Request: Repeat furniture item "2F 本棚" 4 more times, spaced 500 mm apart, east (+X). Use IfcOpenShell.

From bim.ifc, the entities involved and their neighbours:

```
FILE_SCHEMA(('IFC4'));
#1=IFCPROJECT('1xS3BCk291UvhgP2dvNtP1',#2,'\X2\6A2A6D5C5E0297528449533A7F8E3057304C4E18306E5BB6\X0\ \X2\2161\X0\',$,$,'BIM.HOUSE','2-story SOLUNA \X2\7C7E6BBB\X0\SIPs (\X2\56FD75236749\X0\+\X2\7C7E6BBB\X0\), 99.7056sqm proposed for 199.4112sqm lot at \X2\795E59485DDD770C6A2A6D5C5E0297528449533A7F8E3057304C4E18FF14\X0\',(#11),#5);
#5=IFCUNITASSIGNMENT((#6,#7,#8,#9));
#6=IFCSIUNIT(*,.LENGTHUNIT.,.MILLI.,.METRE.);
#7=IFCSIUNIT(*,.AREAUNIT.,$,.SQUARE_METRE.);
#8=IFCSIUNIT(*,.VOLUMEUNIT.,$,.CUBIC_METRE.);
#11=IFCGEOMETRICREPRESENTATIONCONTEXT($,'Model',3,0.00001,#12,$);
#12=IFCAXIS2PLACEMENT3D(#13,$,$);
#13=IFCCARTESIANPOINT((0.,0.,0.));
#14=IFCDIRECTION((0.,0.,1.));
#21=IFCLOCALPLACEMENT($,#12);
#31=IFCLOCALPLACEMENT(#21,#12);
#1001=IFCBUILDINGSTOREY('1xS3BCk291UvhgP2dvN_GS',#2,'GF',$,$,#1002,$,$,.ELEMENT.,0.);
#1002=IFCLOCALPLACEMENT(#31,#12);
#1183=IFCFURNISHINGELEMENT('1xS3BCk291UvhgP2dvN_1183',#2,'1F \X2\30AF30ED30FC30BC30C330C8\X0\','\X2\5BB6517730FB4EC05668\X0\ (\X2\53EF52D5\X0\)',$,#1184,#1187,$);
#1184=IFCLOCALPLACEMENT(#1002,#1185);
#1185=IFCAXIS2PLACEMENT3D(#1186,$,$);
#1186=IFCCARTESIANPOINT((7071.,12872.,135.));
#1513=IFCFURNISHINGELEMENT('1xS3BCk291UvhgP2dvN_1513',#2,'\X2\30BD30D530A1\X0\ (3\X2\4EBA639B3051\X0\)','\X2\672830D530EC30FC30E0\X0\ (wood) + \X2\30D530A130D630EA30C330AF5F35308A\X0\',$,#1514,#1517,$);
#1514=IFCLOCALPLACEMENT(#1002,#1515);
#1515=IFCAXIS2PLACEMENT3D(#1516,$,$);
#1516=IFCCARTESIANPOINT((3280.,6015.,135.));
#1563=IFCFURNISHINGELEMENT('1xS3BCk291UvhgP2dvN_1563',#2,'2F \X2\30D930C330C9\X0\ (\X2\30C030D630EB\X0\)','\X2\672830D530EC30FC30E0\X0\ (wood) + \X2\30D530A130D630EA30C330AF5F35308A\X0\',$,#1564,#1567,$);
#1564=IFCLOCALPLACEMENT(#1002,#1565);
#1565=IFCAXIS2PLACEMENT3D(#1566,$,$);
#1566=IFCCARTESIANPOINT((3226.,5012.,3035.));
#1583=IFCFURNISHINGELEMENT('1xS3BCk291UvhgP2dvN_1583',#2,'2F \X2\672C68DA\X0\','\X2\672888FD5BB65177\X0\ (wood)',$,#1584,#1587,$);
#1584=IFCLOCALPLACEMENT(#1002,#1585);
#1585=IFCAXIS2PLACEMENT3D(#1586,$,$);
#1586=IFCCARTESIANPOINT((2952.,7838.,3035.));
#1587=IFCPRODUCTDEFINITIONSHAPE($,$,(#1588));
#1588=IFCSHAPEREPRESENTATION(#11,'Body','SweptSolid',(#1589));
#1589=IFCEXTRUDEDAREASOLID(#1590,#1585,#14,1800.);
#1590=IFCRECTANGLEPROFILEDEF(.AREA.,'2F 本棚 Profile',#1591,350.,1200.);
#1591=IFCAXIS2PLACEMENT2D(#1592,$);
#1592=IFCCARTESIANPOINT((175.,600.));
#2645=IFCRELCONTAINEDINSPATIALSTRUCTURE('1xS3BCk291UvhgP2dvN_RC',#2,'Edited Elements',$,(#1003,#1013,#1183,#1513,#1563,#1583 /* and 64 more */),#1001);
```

```python
import numpy as np
import ifcopenshell
import ifcopenshell.api.geometry
import ifcopenshell.api.root
import ifcopenshell.util.element
import ifcopenshell.util.placement

model = ifcopenshell.open("bim.ifc")


def reuse_history(source, copy):
    """copy_class also copies each property set's owner history, people and application; keep the originals."""
    for rel in copy.IsDefinedBy:
        if rel.is_a("IfcRelDefinesByProperties") and (history := rel.RelatingPropertyDefinition.OwnerHistory):
            rel.RelatingPropertyDefinition.OwnerHistory = source.OwnerHistory
            ifcopenshell.util.element.remove_deep2(model, history)


source = model.by_guid("1xS3BCk291UvhgP2dvN_1583")
base = ifcopenshell.util.placement.get_local_placement(source.ObjectPlacement)
step = np.array([1.0, 0.0, 0.0]) * 500.0

for i in range(1, 5):
    copy = ifcopenshell.api.root.copy_class(model, product=source)
    copy.Representation = ifcopenshell.util.element.copy_deep(
        model, source.Representation, exclude=["IfcGeometricRepresentationContext", "IfcRepresentationMap"]
    )
    reuse_history(source, copy)
    matrix = base.copy()
    matrix[:3, 3] += i * step
    print("added at", matrix[:3, 3].round(3) + 0.0)
    ifcopenshell.api.geometry.edit_object_placement(model, product=copy, matrix=matrix, is_si=False)

model.write("bim_v2.ifc")
```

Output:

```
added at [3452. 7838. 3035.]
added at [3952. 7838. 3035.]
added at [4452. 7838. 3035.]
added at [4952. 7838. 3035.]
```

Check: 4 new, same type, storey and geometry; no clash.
